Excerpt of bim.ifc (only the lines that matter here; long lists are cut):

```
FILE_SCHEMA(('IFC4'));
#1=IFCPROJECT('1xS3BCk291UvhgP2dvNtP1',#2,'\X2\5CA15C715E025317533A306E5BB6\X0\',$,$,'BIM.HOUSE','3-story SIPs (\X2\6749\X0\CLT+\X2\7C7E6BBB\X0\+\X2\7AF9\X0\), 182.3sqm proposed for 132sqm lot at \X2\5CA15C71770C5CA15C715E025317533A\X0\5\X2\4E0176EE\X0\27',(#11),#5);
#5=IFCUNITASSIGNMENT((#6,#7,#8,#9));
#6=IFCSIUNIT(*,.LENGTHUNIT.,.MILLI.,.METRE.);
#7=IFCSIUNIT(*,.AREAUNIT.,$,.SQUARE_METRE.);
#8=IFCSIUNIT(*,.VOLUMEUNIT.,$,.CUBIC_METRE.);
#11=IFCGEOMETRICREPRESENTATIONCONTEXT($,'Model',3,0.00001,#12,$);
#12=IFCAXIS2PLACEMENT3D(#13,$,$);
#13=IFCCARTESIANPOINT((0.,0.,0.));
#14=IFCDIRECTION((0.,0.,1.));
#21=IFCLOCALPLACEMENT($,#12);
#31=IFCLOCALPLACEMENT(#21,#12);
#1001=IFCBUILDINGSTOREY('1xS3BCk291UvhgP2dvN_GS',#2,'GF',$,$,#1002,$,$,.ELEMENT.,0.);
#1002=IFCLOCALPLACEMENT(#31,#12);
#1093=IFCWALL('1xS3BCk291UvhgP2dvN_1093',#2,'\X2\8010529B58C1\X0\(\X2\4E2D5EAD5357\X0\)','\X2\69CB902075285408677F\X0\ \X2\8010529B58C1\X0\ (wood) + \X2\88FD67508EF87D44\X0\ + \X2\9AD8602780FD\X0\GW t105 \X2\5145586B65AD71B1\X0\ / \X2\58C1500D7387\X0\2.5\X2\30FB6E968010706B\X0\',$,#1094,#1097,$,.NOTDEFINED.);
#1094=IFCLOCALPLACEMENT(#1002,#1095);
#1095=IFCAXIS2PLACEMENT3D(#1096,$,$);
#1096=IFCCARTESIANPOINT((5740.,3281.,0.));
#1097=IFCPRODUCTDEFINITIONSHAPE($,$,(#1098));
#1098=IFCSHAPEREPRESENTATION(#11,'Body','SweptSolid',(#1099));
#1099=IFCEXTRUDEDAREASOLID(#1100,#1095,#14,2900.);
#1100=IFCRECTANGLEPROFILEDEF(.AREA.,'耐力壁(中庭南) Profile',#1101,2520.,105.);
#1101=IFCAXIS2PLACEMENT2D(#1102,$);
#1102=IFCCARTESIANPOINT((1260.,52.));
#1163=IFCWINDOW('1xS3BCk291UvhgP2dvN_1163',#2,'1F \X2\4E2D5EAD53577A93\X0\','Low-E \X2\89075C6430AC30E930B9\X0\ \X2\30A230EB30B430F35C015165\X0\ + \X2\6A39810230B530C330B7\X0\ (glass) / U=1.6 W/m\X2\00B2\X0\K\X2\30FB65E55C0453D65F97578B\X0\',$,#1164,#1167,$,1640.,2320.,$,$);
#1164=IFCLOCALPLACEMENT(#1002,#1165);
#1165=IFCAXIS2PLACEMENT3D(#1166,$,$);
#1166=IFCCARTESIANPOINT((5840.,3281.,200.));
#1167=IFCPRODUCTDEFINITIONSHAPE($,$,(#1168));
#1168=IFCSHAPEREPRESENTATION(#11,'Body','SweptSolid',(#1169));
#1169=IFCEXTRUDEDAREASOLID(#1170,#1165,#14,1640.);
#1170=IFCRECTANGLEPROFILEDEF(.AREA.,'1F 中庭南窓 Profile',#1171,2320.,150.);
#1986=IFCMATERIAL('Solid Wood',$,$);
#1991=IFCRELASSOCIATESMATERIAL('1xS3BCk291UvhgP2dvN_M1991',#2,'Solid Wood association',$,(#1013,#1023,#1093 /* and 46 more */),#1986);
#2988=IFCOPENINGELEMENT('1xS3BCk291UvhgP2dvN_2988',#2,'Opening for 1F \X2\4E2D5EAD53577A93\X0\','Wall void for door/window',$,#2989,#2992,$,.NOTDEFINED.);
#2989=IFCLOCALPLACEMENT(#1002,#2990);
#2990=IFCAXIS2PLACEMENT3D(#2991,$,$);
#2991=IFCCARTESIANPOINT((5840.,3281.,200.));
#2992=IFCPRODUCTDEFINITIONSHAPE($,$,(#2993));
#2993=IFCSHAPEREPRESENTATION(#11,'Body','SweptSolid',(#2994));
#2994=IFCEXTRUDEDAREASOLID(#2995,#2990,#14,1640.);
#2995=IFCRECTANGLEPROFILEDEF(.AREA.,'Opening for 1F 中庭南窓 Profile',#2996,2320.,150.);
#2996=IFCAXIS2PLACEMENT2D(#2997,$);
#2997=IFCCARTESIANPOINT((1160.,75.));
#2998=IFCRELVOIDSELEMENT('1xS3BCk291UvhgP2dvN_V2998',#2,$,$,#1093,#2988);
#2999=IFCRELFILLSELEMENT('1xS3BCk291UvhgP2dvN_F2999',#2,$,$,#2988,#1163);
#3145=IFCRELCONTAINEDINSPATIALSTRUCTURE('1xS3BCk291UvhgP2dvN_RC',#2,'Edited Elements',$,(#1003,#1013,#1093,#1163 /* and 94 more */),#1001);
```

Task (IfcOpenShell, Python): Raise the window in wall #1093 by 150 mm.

```python
import numpy as np
import ifcopenshell
import ifcopenshell.api.geometry
import ifcopenshell.util.placement
import ifcopenshell.util.unit

model = ifcopenshell.open("bim.ifc")
unit_scale = ifcopenshell.util.unit.calculate_unit_scale(model)

window = model.by_guid("1xS3BCk291UvhgP2dvN_1163")
opening = window.FillsVoids[0].RelatingOpeningElement
dz = 0.15 / unit_scale

shift = np.array([0.0, 0.0, dz])
# The window is not placed relative to its opening, so move both.
for product in (opening, window):
    matrix = ifcopenshell.util.placement.get_local_placement(product.ObjectPlacement)
    matrix[:3, 3] += shift
    ifcopenshell.api.geometry.edit_object_placement(model, product=product, matrix=matrix, is_si=False)

print(f"moved by {dz * unit_scale:+.3f} m")

model.write("bim_rev.ifc")
```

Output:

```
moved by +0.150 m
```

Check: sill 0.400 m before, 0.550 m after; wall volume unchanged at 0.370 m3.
